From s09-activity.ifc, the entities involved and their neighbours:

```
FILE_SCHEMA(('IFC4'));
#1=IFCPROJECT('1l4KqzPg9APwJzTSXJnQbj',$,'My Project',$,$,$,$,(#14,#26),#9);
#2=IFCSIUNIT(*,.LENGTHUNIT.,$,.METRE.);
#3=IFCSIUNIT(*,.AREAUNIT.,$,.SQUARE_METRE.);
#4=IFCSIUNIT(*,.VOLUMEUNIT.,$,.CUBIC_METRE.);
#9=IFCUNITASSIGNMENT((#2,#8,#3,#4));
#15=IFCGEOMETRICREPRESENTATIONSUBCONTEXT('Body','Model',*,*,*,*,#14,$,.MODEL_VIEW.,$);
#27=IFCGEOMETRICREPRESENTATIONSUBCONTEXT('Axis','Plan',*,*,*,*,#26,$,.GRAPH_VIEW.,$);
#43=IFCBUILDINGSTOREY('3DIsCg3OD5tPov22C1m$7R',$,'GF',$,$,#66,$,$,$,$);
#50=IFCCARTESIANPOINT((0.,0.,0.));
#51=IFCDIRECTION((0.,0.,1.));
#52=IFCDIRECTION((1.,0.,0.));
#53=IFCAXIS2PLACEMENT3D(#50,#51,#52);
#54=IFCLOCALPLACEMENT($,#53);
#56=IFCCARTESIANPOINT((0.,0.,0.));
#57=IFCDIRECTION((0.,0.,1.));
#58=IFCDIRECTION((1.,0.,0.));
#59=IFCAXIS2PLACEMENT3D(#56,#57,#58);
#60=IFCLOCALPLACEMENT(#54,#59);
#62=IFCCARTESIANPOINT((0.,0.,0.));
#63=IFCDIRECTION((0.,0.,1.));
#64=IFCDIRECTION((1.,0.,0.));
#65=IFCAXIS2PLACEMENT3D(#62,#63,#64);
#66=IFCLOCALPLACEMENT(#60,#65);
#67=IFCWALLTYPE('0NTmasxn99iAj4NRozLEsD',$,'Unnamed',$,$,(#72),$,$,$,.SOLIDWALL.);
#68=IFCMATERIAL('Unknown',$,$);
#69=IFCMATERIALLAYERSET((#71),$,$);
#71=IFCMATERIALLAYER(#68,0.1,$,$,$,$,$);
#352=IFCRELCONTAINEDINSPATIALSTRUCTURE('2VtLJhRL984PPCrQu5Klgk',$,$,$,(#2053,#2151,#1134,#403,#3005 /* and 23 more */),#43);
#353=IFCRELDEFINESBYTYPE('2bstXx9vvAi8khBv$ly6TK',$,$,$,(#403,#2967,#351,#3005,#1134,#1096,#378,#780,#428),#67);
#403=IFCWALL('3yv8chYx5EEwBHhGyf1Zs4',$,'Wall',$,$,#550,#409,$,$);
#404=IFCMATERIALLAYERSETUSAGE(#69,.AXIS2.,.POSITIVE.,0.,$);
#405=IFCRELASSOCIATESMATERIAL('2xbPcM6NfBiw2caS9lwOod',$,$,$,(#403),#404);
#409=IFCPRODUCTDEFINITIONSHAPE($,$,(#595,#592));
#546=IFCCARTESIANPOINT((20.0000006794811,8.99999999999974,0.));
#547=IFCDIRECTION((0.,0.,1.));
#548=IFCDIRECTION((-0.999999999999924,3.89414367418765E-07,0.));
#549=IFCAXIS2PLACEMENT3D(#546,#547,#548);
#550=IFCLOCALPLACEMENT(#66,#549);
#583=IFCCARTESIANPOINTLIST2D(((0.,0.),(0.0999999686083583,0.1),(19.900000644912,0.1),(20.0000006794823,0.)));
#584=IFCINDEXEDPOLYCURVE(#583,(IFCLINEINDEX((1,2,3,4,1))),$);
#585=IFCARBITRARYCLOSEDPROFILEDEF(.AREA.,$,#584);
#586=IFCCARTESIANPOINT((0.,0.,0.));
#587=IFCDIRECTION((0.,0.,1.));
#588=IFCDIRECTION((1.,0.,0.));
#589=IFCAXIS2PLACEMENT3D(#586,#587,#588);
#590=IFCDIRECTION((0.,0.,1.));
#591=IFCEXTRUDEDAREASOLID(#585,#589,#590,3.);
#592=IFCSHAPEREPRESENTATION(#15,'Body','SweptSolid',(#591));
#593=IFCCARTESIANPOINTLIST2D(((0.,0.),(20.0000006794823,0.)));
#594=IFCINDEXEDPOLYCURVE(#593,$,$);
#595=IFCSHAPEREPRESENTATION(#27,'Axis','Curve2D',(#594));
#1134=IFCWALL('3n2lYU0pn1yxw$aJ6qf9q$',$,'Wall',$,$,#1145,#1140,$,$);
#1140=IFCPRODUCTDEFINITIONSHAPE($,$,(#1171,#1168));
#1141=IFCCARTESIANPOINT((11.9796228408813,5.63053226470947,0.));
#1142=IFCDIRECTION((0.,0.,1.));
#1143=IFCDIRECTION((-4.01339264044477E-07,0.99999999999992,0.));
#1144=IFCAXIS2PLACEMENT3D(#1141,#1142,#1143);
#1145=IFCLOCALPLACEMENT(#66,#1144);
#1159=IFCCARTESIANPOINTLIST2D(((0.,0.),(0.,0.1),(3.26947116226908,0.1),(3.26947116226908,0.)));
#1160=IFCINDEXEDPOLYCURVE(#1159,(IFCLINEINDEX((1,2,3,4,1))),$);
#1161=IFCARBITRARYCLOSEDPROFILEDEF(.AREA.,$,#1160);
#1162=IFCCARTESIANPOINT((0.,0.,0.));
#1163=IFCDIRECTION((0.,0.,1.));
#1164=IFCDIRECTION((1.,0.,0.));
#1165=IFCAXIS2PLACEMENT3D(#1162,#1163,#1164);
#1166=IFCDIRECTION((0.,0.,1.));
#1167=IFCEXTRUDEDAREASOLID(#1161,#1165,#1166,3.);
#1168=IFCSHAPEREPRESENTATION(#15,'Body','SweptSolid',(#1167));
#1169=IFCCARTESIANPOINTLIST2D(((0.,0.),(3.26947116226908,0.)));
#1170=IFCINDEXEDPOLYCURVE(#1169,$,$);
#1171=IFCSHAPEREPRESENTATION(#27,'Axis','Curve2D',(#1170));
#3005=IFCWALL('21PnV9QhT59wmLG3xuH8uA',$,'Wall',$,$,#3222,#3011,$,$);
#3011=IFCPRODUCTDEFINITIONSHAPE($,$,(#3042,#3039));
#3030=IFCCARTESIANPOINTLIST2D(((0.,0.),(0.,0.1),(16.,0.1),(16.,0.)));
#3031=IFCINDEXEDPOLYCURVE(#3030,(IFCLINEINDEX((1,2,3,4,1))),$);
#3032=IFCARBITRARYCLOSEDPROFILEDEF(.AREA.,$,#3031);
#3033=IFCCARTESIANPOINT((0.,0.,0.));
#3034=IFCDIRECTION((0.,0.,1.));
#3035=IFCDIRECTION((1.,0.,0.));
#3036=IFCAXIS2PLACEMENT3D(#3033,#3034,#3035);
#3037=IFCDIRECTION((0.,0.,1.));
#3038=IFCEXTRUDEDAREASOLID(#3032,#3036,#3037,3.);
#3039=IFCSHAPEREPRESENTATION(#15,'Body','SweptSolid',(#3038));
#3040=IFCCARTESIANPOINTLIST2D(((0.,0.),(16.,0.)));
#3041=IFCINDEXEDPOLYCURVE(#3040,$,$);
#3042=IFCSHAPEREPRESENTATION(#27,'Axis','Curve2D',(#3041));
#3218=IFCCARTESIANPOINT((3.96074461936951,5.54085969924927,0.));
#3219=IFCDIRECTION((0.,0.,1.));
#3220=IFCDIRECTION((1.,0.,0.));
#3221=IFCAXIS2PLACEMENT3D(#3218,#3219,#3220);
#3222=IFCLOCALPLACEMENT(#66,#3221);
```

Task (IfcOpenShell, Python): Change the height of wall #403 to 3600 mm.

```python
import ifcopenshell
import ifcopenshell.geom
import ifcopenshell.util.representation
import ifcopenshell.util.shape
import ifcopenshell.util.unit

model = ifcopenshell.open("s09-activity.ifc")
unit_scale = ifcopenshell.util.unit.calculate_unit_scale(model)
settings = ifcopenshell.geom.settings()


def volume(element):
    """Net volume in cubic metres, openings subtracted."""
    shape = ifcopenshell.geom.create_shape(settings, element)
    return ifcopenshell.util.shape.get_volume(shape.geometry)


wall = model.by_guid("3yv8chYx5EEwBHhGyf1Zs4")
before = volume(wall)

body = ifcopenshell.util.representation.get_representation(wall, "Model", "Body")
solid = body.Items[0]
old_height = solid.Depth
solid.Depth = 3.6 / unit_scale
after = volume(wall)

print(f"height {old_height:g} -> {solid.Depth:g}, volume {before:.3f} -> {after:.3f} m3")

model.write("s09-activity_rev.ifc")
```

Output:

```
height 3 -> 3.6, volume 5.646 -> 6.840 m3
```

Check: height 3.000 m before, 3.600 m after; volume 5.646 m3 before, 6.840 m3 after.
